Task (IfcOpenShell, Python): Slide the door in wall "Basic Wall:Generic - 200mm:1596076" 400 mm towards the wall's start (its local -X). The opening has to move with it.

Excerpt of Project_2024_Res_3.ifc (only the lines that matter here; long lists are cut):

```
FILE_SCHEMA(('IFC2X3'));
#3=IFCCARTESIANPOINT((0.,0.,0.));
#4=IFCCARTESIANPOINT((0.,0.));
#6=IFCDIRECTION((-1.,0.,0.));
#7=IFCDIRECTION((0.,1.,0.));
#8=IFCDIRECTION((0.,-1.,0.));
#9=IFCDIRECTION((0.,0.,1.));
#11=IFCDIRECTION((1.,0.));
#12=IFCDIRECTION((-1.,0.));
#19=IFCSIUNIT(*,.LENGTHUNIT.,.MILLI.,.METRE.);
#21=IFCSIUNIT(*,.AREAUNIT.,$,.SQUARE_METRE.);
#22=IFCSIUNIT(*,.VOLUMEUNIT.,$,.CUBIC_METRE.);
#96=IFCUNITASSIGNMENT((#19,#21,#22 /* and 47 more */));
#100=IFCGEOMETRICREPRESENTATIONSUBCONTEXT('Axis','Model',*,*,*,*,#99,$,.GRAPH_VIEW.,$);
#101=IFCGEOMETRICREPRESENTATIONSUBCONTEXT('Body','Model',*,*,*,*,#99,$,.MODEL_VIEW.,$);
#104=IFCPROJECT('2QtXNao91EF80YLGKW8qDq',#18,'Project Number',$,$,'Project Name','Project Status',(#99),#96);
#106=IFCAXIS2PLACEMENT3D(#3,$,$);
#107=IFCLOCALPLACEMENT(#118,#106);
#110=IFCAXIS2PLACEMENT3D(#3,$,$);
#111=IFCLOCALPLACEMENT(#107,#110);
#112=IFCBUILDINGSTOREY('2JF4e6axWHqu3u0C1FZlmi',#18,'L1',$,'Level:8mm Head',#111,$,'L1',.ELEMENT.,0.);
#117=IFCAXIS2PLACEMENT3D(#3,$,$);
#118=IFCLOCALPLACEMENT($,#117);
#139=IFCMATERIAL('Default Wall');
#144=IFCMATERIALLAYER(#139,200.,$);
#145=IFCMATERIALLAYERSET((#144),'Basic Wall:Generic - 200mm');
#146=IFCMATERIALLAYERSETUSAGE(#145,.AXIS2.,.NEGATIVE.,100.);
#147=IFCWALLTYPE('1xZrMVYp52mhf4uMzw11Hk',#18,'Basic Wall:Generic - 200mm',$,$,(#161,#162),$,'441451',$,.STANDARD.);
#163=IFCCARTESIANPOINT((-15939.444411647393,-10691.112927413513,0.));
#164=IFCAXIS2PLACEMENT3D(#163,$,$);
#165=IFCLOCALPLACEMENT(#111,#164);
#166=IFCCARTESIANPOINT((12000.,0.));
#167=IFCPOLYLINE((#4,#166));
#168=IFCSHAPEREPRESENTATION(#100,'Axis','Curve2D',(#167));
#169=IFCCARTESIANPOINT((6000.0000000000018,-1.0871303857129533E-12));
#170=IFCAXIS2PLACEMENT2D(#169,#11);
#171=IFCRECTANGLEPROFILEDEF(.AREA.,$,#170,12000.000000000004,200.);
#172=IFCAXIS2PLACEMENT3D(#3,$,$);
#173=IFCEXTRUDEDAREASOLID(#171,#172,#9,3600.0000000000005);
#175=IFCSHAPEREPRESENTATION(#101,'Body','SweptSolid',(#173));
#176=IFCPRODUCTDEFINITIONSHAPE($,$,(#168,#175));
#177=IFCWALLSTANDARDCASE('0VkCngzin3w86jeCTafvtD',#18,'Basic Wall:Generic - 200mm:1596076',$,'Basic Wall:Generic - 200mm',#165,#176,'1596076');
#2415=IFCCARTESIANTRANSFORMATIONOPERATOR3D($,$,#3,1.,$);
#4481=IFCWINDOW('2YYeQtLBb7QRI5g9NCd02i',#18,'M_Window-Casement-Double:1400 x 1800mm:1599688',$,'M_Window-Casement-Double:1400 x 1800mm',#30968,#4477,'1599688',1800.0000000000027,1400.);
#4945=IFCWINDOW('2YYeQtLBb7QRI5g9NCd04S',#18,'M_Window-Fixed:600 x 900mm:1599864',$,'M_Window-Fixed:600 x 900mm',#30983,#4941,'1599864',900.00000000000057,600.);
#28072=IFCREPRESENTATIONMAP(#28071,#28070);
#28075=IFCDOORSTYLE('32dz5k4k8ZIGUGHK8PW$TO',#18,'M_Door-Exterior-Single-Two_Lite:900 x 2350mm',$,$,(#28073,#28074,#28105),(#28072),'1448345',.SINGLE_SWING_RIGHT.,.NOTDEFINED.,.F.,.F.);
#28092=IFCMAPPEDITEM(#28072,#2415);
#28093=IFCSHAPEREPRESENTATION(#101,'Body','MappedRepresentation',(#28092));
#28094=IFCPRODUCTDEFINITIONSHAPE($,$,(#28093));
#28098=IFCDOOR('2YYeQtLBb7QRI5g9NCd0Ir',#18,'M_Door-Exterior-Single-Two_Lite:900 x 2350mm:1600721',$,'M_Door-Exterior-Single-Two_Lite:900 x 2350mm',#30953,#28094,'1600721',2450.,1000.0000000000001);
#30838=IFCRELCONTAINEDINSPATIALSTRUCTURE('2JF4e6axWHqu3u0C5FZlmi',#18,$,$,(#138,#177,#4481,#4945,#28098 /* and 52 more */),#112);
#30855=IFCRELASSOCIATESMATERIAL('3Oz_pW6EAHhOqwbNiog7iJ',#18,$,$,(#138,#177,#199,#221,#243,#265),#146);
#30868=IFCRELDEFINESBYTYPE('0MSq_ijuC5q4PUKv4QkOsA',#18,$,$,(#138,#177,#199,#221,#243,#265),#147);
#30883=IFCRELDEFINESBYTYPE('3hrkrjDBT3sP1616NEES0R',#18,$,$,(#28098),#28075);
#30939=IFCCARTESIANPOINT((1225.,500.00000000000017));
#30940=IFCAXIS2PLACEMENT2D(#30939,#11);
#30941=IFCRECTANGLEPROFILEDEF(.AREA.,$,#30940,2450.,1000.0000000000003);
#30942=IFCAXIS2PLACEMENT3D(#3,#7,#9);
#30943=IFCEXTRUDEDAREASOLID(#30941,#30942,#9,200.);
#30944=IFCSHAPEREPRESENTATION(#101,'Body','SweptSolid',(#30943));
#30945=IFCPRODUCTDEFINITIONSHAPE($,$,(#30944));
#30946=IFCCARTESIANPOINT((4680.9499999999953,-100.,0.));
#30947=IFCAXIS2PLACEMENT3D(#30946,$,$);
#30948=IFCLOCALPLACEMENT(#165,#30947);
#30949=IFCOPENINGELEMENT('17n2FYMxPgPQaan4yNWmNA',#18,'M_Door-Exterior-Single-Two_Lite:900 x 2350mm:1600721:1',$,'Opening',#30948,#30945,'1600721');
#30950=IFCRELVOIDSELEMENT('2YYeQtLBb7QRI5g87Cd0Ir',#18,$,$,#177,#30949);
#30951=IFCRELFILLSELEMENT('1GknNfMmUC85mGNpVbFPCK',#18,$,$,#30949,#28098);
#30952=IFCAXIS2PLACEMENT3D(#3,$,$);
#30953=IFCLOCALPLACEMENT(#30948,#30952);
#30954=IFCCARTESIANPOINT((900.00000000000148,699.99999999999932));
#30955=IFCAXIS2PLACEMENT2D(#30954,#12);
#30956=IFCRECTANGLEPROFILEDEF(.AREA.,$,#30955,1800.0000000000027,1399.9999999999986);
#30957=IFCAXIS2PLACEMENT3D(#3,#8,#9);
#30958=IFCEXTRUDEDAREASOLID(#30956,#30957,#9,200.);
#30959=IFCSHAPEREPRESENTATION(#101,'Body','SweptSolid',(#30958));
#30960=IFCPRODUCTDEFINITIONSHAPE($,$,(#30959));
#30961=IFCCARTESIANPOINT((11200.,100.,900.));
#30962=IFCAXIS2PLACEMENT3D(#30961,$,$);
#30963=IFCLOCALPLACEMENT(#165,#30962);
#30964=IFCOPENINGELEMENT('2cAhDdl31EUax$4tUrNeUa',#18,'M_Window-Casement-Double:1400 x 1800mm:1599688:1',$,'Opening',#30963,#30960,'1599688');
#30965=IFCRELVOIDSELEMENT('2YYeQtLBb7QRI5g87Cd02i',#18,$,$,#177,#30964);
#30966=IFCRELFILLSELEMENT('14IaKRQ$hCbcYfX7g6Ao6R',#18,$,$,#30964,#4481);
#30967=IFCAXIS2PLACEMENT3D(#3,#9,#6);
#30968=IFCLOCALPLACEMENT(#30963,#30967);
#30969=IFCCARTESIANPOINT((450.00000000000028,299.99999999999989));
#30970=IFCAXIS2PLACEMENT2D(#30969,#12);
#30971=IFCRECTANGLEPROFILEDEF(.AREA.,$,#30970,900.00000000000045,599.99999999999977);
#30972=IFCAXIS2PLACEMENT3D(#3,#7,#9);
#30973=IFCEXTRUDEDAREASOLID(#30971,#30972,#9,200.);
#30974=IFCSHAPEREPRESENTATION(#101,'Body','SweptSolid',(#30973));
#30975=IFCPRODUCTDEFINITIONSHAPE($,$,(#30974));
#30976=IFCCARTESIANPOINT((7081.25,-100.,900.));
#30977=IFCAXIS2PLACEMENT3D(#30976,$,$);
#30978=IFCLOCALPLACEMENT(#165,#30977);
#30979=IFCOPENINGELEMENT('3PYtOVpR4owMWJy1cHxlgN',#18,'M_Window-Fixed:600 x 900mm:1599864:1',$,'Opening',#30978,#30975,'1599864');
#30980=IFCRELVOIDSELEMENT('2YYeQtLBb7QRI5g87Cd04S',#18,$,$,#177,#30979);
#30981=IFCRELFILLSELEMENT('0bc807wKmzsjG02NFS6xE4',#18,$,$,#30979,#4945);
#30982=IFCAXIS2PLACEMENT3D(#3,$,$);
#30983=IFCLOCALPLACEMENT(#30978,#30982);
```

```python
import ifcopenshell
import ifcopenshell.api.geometry
import ifcopenshell.util.placement

model = ifcopenshell.open("Project_2024_Res_3.ifc")

door = model.by_id(28098)
opening = door.FillsVoids[0].RelatingOpeningElement
wall = opening.VoidsElements[0].RelatingBuildingElement

wall_matrix = ifcopenshell.util.placement.get_local_placement(wall.ObjectPlacement)
shift = wall_matrix[:3, 0] * -400.0
before = ifcopenshell.util.placement.get_local_placement(door.ObjectPlacement)[:3, 3].copy()

# The door is placed relative to its opening, so it follows when the opening moves.
matrix = ifcopenshell.util.placement.get_local_placement(opening.ObjectPlacement)
matrix[:3, 3] += shift
ifcopenshell.api.geometry.edit_object_placement(
    model, product=opening, matrix=matrix, is_si=False, should_transform_children=True
)

after = ifcopenshell.util.placement.get_local_placement(door.ObjectPlacement)[:3, 3]
print("door moved by", (after - before).round(3) + 0.0)

model.write("Project_2024_Res_3_v2.ifc")
```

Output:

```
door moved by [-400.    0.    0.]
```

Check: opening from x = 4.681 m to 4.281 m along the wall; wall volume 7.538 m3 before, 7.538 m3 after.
